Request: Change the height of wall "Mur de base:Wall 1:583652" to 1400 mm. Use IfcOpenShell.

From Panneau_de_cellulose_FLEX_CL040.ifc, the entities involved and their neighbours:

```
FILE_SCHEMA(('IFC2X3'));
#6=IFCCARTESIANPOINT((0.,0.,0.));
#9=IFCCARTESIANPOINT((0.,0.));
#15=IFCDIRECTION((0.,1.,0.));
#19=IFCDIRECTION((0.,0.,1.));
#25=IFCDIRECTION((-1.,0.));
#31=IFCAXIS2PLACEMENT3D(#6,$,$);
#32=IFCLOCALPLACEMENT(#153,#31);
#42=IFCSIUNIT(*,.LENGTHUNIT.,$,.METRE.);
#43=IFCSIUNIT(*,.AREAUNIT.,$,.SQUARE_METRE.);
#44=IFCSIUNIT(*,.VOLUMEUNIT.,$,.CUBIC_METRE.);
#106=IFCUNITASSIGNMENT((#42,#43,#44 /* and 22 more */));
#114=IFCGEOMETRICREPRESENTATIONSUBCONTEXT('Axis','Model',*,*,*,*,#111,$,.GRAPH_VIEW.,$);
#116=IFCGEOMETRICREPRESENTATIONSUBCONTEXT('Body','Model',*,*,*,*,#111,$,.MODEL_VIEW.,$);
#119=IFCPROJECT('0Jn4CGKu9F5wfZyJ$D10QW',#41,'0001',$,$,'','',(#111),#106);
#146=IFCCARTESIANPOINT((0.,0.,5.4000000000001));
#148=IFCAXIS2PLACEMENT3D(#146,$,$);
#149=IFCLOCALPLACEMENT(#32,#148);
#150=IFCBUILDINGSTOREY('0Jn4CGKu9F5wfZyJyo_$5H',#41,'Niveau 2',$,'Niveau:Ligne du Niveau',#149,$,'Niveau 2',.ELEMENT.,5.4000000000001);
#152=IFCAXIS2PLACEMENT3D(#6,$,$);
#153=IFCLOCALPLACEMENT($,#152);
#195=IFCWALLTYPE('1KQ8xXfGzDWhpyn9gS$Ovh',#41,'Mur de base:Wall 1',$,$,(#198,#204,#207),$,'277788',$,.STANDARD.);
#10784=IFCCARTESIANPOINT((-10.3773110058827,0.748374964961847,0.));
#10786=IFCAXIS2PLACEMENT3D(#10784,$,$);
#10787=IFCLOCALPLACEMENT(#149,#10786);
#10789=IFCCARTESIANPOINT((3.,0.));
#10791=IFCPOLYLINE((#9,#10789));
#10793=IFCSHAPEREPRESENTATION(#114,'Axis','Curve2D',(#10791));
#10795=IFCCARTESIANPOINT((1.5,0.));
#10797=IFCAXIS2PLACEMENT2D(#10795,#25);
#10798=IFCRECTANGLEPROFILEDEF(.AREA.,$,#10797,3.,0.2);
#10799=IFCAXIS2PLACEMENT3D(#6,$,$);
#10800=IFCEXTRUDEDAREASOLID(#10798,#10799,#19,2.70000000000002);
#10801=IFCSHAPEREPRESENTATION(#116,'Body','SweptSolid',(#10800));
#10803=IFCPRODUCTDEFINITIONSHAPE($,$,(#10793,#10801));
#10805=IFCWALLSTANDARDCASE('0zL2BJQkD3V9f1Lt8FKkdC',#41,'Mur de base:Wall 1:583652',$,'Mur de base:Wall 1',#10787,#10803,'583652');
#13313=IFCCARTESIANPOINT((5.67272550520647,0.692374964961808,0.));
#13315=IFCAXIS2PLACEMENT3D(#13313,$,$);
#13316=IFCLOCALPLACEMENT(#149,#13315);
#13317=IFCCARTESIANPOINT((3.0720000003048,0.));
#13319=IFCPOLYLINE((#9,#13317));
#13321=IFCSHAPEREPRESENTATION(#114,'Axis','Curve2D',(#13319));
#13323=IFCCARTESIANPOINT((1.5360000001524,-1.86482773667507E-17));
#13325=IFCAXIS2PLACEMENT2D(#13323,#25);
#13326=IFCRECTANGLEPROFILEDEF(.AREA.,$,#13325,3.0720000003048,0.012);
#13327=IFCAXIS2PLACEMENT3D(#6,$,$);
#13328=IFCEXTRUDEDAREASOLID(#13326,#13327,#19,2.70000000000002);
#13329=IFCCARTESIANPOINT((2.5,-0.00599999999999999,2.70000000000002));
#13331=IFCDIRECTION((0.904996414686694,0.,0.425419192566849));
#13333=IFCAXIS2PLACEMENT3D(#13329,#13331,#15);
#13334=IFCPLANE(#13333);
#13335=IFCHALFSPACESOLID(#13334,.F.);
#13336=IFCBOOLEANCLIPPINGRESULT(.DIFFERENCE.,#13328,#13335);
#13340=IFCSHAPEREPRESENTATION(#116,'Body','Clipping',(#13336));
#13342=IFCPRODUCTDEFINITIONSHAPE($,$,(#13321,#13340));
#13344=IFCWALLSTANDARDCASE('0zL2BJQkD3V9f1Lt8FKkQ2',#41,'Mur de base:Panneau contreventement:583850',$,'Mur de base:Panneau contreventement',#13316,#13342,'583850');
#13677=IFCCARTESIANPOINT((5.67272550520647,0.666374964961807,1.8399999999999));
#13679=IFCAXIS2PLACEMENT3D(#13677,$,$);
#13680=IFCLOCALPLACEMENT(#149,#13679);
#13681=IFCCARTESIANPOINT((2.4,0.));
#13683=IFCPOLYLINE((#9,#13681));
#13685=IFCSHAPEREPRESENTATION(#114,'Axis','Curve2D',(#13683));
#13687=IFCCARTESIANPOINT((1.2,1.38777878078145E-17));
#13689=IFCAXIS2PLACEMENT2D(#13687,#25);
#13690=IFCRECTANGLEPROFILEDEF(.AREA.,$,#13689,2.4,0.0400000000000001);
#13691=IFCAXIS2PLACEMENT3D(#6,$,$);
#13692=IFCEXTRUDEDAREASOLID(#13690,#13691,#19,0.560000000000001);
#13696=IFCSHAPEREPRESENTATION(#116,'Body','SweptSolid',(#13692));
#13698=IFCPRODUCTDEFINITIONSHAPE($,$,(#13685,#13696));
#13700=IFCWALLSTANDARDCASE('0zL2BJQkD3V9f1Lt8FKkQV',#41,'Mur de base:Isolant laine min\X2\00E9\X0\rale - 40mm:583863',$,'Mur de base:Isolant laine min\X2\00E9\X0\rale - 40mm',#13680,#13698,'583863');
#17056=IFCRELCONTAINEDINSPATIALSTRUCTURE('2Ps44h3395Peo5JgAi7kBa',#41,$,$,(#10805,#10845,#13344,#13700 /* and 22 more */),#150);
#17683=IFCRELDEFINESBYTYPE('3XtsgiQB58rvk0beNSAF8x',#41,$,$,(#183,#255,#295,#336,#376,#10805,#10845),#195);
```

```python
import ifcopenshell
import ifcopenshell.geom
import ifcopenshell.util.representation
import ifcopenshell.util.shape
import ifcopenshell.util.unit

model = ifcopenshell.open("Panneau_de_cellulose_FLEX_CL040.ifc")
unit_scale = ifcopenshell.util.unit.calculate_unit_scale(model)
settings = ifcopenshell.geom.settings()


def volume(element):
    """Net volume in cubic metres, openings subtracted."""
    shape = ifcopenshell.geom.create_shape(settings, element)
    return ifcopenshell.util.shape.get_volume(shape.geometry)


wall = model.by_guid("0zL2BJQkD3V9f1Lt8FKkdC")
before = volume(wall)

body = ifcopenshell.util.representation.get_representation(wall, "Model", "Body")
solid = body.Items[0]
old_height = solid.Depth
solid.Depth = 1.4 / unit_scale
after = volume(wall)

print(f"height {old_height:g} -> {solid.Depth:g}, volume {before:.3f} -> {after:.3f} m3")

model.write("Panneau_de_cellulose_FLEX_CL040_updated.ifc")
```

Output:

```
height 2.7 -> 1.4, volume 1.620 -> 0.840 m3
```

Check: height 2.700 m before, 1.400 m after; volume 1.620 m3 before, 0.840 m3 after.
